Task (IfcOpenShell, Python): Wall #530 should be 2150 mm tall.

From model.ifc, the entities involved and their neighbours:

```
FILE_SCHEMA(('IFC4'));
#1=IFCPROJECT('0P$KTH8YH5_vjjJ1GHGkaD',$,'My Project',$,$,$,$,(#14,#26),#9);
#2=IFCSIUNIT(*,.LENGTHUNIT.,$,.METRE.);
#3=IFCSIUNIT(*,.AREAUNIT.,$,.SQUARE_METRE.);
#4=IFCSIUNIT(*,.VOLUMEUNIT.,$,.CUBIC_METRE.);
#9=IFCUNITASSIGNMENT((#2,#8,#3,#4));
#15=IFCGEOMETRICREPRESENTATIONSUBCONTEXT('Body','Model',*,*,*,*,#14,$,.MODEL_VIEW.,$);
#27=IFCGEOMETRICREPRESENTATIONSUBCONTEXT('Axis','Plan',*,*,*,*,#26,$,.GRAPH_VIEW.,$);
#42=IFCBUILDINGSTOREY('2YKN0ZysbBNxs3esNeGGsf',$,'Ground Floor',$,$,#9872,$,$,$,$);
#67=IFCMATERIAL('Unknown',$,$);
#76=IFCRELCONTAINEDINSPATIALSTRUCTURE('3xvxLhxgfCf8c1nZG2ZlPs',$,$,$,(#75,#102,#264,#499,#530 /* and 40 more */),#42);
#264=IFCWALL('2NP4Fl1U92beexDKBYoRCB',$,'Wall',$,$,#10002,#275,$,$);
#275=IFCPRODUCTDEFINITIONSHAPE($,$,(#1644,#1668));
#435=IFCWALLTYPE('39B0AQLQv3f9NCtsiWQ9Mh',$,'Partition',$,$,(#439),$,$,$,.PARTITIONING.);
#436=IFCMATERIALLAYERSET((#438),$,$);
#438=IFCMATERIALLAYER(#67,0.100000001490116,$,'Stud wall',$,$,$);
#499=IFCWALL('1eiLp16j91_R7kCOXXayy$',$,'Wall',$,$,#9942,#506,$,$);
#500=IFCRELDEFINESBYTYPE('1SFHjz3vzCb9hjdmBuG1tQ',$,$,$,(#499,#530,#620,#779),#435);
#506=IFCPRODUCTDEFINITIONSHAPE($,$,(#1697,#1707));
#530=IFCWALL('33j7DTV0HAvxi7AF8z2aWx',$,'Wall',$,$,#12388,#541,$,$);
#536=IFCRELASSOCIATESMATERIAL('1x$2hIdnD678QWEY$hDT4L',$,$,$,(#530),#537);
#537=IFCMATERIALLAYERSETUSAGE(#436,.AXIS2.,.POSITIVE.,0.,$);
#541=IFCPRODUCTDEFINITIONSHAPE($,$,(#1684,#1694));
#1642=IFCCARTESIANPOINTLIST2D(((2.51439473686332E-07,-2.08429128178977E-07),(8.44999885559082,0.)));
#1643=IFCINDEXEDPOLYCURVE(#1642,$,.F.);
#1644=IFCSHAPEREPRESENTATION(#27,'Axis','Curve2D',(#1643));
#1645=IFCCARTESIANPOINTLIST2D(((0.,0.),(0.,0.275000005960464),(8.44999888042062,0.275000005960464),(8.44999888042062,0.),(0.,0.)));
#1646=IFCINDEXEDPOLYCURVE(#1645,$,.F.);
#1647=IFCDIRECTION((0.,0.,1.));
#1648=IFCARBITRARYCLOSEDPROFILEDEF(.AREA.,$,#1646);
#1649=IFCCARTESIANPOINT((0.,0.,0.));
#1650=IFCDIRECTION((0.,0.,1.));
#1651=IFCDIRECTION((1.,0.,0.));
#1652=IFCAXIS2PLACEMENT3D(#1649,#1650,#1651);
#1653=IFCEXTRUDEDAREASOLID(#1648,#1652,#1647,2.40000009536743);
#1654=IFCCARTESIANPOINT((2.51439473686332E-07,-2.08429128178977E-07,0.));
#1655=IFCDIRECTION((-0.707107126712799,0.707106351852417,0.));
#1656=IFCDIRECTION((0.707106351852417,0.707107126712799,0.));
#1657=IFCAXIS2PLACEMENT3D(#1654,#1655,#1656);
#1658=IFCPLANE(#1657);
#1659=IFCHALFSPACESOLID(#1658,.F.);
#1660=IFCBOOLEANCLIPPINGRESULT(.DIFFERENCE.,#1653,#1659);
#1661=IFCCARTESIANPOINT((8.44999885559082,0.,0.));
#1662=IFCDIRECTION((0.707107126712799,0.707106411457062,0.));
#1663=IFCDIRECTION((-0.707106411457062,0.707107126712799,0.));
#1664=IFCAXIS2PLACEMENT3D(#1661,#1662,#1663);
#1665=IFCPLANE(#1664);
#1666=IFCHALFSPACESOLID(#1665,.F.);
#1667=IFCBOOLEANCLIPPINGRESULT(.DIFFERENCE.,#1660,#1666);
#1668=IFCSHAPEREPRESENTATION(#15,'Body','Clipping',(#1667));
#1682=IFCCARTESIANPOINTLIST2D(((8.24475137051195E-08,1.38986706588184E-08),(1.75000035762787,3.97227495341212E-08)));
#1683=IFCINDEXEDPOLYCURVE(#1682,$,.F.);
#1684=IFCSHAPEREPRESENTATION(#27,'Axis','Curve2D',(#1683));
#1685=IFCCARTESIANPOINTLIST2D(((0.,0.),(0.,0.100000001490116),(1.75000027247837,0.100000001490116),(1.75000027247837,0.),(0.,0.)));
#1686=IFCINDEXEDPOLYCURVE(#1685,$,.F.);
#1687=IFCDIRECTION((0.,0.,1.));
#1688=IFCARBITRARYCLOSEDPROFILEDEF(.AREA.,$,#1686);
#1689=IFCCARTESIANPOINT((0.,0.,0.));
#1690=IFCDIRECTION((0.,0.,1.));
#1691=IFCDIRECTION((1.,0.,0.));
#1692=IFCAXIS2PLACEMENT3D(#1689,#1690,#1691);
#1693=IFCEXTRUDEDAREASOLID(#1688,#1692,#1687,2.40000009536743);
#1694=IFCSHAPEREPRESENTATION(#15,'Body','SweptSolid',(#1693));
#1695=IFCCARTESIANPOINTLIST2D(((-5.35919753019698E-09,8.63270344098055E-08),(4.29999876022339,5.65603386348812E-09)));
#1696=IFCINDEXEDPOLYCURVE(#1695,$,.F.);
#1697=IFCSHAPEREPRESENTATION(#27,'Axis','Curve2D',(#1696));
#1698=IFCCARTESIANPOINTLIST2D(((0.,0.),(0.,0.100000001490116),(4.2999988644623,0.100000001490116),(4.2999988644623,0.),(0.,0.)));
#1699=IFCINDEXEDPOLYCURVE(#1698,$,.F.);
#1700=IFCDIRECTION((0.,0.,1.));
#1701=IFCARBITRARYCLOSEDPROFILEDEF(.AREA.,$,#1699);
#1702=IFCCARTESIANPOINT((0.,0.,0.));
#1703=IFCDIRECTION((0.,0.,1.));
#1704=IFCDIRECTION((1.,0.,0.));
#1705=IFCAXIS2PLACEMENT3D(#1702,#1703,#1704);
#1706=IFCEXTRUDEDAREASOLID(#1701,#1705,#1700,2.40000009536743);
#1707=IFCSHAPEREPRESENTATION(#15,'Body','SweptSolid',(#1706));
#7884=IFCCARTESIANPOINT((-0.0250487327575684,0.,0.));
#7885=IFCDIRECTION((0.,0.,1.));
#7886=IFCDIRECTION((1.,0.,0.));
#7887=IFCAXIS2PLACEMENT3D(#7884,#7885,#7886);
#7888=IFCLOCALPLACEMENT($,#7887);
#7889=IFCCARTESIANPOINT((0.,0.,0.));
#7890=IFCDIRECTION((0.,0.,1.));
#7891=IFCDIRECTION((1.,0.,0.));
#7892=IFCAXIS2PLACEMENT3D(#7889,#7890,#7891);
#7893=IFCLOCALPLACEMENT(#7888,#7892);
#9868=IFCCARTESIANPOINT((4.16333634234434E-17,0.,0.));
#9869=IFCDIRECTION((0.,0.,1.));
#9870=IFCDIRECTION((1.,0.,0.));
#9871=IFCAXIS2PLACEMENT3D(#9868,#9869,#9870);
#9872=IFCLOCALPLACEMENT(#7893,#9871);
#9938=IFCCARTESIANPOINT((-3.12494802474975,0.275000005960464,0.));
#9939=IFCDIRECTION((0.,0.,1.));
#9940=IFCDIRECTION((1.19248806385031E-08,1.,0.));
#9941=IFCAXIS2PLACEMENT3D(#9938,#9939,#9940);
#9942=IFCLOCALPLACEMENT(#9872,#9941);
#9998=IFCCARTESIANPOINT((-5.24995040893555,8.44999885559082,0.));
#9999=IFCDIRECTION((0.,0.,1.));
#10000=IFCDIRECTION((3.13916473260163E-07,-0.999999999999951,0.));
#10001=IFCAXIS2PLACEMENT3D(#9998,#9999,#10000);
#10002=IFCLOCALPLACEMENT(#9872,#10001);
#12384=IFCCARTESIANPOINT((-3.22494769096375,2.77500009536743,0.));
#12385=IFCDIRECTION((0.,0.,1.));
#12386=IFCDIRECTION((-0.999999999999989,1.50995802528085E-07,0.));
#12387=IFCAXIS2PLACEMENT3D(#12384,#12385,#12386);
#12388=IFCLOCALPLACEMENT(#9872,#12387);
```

```python
import ifcopenshell
import ifcopenshell.geom
import ifcopenshell.util.representation
import ifcopenshell.util.shape

model = ifcopenshell.open("model.ifc")
settings = ifcopenshell.geom.settings()


def volume(element):
    """Net volume in cubic metres, openings subtracted."""
    shape = ifcopenshell.geom.create_shape(settings, element)
    return ifcopenshell.util.shape.get_volume(shape.geometry)


wall = model.by_guid("33j7DTV0HAvxi7AF8z2aWx")
before = volume(wall)

body = ifcopenshell.util.representation.get_representation(wall, "Model", "Body")
solid = body.Items[0]
old_height = solid.Depth
solid.Depth = 2.15
after = volume(wall)

print(f"height {old_height:g} -> {solid.Depth:g}, volume {before:.3f} -> {after:.3f} m3")

model.write("model_v2.ifc")
```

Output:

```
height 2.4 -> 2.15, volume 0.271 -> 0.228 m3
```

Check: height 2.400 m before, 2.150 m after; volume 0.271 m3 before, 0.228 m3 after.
